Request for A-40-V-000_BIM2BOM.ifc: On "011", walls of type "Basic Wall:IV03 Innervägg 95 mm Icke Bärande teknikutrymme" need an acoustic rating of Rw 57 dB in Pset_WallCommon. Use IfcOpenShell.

First a look at what the model holds.

```python
import ifcopenshell
import ifcopenshell.util.element

model = ifcopenshell.open("A-40-V-000_BIM2BOM.ifc")
print(model.schema)
storey = next(s for s in model.by_type("IfcBuildingStorey") if s.Name == "011")
walls = [e for e in ifcopenshell.util.element.get_decomposition(storey) if e.is_a("IfcWall")]
seen = {}
for e in walls:
    element_type = ifcopenshell.util.element.get_type(e)
    key = (element_type.Name if element_type != e and element_type else None, ifcopenshell.util.element.get_pset(e, "Pset_WallCommon", "AcousticRating"))
    seen[key] = seen.get(key, 0) + 1
for (name, value), count in sorted(seen.items(), key=str):
    print(count, "x", name, "|", value)
```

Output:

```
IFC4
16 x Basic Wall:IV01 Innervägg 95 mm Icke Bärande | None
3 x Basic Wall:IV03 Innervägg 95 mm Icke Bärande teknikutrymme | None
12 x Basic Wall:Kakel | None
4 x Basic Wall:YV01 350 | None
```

```python
import ifcopenshell
import ifcopenshell.api.pset
import ifcopenshell.util.element

model = ifcopenshell.open("A-40-V-000_BIM2BOM.ifc")

storey = next(s for s in model.by_type("IfcBuildingStorey") if s.Name == "011")
walls = [e for e in ifcopenshell.util.element.get_decomposition(storey) if e.is_a("IfcWall")]

count = 0
for e in walls:
    element_type = ifcopenshell.util.element.get_type(e)
    if element_type in (None, e) or element_type.Name != "Basic Wall:IV03 Innervägg 95 mm Icke Bärande teknikutrymme":
        continue
    # add_pset returns the element's existing set when there is one.
    pset = ifcopenshell.api.pset.add_pset(model, product=e, name="Pset_WallCommon")
    ifcopenshell.api.pset.edit_pset(model, pset=pset, properties={"AcousticRating": "Rw 57 dB"})
    count += 1

print(count, "walls updated")

model.write("A-40-V-000_BIM2BOM_updated.ifc")
```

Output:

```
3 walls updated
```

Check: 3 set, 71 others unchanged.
